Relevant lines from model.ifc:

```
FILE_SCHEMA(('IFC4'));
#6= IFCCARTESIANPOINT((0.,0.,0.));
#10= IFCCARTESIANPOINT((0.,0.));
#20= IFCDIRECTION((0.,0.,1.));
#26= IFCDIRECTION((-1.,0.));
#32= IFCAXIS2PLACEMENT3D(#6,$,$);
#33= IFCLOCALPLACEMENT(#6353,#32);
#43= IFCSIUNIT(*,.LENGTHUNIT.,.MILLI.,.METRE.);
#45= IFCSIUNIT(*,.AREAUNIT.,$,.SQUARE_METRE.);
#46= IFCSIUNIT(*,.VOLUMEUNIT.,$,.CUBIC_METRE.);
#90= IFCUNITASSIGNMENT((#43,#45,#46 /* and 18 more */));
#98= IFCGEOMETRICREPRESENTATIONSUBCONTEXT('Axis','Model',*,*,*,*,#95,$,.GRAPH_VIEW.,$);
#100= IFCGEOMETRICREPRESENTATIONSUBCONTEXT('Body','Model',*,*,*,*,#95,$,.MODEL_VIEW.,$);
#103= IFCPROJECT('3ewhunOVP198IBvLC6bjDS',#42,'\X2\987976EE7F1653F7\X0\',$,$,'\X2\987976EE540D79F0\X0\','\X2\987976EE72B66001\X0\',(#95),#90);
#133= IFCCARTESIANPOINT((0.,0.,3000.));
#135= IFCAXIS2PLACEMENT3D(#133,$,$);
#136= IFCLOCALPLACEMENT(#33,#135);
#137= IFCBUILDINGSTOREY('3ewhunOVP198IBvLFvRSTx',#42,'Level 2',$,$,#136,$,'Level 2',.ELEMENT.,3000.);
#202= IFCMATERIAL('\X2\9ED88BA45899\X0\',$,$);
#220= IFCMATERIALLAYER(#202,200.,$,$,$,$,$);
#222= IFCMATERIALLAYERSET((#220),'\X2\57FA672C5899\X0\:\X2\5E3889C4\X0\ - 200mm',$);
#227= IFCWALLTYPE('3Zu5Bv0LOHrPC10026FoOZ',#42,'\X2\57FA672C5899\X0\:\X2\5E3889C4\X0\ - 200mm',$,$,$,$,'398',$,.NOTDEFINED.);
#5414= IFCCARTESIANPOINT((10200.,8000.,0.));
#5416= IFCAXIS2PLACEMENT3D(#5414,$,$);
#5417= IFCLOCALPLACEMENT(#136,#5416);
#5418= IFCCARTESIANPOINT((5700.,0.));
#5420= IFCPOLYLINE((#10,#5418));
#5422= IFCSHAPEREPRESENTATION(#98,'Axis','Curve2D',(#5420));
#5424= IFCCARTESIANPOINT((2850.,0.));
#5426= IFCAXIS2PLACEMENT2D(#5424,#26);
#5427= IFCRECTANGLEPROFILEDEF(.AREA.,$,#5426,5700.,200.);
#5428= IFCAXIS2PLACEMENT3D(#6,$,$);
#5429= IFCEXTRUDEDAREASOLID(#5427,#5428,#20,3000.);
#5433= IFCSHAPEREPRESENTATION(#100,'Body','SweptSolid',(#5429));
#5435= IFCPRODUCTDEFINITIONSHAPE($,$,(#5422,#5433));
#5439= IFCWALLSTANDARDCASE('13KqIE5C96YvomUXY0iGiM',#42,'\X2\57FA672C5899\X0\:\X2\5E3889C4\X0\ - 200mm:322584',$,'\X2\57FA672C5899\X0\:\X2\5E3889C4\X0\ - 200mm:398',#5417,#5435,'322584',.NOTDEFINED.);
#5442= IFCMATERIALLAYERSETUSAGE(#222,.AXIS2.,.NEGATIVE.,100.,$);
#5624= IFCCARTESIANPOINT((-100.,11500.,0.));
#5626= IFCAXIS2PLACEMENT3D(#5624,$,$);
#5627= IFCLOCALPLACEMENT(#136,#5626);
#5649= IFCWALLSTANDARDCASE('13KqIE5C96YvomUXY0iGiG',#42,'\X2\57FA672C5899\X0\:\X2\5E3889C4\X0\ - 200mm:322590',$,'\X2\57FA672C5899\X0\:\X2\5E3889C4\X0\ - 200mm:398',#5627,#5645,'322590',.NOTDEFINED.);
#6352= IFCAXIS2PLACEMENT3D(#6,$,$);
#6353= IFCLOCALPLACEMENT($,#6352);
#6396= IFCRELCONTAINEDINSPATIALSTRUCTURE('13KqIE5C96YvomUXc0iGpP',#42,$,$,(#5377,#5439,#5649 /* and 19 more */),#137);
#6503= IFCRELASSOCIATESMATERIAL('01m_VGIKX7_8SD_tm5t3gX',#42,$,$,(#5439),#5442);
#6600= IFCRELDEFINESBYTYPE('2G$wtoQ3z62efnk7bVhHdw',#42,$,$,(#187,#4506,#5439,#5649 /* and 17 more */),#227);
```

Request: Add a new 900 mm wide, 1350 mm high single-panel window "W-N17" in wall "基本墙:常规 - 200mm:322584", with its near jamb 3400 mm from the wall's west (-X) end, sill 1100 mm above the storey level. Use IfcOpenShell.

```python
import numpy as np
import ifcopenshell
import ifcopenshell.api.feature
import ifcopenshell.api.geometry
import ifcopenshell.api.root
import ifcopenshell.api.spatial
import ifcopenshell.geom
import ifcopenshell.util.element
import ifcopenshell.util.placement
import ifcopenshell.util.representation
import ifcopenshell.util.shape
import ifcopenshell.util.unit

model = ifcopenshell.open("model.ifc")
unit_scale = ifcopenshell.util.unit.calculate_unit_scale(model)
settings = ifcopenshell.geom.settings()


def volume(element):
    """Net volume in cubic metres, openings subtracted."""
    shape = ifcopenshell.geom.create_shape(settings, element)
    return ifcopenshell.util.shape.get_volume(shape.geometry)


wall = model.by_id(5439)
storey = ifcopenshell.util.element.get_container(wall, ifc_class="IfcBuildingStorey")
context = ifcopenshell.util.representation.get_context(model, "Model", "Body", "MODEL_VIEW")
before = volume(wall)

width, height, from_end, sill = 0.9, 1.35, 3.4, 1.1  # metres

# The wall runs along its own X axis, and the end named is its -X end.
wall_shape = ifcopenshell.geom.create_shape(settings, wall)
x, y, z = ifcopenshell.util.shape.get_vertices(wall_shape.geometry).T
start = x.min() + from_end
face, thickness = float(y.min()), float(y.max() - y.min())
wall_matrix = ifcopenshell.util.placement.get_local_placement(wall.ObjectPlacement)
level = ifcopenshell.util.placement.get_local_placement(storey.ObjectPlacement)[2, 3]


def in_wall(x, y):
    """Placement at x, y metres in the wall's axes, at sill height."""
    matrix = wall_matrix.copy()
    matrix[:, 3] = wall_matrix @ np.array([x / unit_scale, y / unit_scale, 0.0, 1.0])
    matrix[2, 3] = level + sill / unit_scale
    return matrix


# Opening: a box that overshoots both wall faces by 50 mm.
opening = ifcopenshell.api.root.create_entity(model, ifc_class="IfcOpeningElement", predefined_type="OPENING")
box = ifcopenshell.api.geometry.add_wall_representation(
    model, context=context, length=width, height=height, thickness=thickness + 0.1
)
ifcopenshell.api.geometry.assign_representation(model, product=opening, representation=box)
ifcopenshell.api.geometry.edit_object_placement(model, product=opening, matrix=in_wall(start, face - 0.05), is_si=False)
ifcopenshell.api.feature.add_feature(model, feature=opening, element=wall)

window = ifcopenshell.api.root.create_entity(model, ifc_class="IfcWindow", name="W-N17", predefined_type="WINDOW")
window.OverallWidth, window.OverallHeight = width / unit_scale, height / unit_scale
window.PartitioningType = "SINGLE_PANEL"
body = ifcopenshell.api.geometry.add_window_representation(
    model,
    context=context,
    overall_width=window.OverallWidth,
    overall_height=window.OverallHeight,
    partition_type="SINGLE_PANEL",
)
ifcopenshell.api.geometry.assign_representation(model, product=window, representation=body)
ifcopenshell.api.spatial.assign_container(model, products=[window], relating_structure=storey)
ifcopenshell.api.feature.add_filling(model, opening=opening, element=window)

# Centre the window in the wall's thickness.
ifcopenshell.api.geometry.edit_object_placement(model, product=window, matrix=in_wall(start, face), is_si=False)
window_shape = ifcopenshell.geom.create_shape(settings, window)
depth = ifcopenshell.util.shape.get_vertices(window_shape.geometry)[:, 1]
offset = face + thickness / 2 - (depth.min() + depth.max()) / 2
ifcopenshell.api.geometry.edit_object_placement(model, product=window, matrix=in_wall(start, offset), is_si=False)

after = volume(wall)

print(f"wall volume {before:.3f} -> {after:.3f} m3")

model.write("model-out.ifc")
```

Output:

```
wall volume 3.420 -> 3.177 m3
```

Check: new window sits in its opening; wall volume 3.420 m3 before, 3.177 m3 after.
